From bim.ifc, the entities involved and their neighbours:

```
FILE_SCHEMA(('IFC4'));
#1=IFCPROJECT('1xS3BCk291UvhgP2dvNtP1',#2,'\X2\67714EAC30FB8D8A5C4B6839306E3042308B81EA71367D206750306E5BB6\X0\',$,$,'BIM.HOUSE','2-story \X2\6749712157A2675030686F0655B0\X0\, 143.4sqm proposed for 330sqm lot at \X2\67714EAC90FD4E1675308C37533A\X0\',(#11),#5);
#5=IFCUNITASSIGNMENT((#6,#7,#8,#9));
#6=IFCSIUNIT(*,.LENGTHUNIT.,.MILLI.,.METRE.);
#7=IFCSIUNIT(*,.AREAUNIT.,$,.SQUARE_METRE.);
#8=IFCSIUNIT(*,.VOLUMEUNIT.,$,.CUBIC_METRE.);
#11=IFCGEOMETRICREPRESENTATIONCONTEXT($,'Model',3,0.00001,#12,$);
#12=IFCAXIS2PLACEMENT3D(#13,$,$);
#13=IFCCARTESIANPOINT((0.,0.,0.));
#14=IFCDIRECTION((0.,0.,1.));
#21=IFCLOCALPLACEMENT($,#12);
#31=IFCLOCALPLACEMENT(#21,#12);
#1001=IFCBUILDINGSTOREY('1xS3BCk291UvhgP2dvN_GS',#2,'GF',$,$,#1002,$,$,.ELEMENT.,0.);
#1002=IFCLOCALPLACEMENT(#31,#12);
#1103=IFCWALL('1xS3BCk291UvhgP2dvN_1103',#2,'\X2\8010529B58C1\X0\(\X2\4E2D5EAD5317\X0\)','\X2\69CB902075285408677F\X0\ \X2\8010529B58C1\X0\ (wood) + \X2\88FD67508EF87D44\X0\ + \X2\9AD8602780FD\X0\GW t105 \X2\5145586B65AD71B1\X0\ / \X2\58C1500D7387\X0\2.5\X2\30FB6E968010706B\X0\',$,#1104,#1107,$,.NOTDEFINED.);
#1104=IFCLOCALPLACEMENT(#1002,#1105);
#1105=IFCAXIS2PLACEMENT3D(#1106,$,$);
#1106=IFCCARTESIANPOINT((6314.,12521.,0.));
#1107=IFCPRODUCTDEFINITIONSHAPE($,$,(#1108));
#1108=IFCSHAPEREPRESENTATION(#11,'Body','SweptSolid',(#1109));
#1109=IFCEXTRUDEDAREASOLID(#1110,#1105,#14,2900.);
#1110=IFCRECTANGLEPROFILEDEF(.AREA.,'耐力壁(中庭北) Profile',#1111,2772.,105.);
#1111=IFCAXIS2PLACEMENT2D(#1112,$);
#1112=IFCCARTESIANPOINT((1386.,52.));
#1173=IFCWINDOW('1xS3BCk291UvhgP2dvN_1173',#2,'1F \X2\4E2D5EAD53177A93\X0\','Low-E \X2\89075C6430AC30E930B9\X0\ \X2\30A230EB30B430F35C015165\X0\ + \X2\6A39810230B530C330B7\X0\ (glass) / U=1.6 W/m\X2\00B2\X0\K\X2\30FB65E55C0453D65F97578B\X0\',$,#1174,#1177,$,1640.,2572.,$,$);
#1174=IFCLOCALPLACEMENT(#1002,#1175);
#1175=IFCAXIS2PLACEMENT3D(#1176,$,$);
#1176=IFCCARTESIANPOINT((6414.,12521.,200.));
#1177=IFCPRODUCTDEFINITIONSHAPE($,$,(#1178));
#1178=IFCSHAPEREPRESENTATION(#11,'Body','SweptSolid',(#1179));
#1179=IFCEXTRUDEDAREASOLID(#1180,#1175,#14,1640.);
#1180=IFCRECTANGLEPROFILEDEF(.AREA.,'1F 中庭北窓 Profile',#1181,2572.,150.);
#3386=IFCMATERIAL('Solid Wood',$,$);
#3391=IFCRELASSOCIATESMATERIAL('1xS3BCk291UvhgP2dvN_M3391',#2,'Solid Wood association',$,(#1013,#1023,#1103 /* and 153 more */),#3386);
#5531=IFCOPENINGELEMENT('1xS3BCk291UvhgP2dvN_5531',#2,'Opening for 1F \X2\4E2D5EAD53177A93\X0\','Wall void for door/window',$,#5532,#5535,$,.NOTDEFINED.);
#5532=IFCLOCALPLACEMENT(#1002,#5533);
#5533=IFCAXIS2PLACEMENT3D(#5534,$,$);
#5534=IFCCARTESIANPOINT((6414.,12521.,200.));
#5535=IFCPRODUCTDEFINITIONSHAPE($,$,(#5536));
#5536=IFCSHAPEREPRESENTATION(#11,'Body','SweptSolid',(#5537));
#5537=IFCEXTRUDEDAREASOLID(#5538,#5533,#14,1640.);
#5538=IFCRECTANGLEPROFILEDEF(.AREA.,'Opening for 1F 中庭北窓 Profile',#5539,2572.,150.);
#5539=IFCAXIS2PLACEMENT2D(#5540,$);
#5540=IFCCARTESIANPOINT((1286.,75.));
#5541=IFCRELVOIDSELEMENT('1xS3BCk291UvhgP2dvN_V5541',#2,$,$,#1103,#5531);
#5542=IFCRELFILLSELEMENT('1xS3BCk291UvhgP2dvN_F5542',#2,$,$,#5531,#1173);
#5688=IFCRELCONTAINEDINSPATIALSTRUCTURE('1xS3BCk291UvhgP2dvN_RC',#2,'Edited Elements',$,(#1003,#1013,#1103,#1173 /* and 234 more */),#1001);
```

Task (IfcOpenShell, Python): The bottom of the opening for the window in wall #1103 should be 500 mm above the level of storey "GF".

```python
import numpy as np
import ifcopenshell
import ifcopenshell.api.geometry
import ifcopenshell.geom
import ifcopenshell.util.element
import ifcopenshell.util.placement
import ifcopenshell.util.shape
import ifcopenshell.util.unit

model = ifcopenshell.open("bim.ifc")
unit_scale = ifcopenshell.util.unit.calculate_unit_scale(model)

window = model.by_guid("1xS3BCk291UvhgP2dvN_1173")
opening = window.FillsVoids[0].RelatingOpeningElement
storey = ifcopenshell.util.element.get_container(window, ifc_class="IfcBuildingStorey")
level = ifcopenshell.util.placement.get_local_placement(storey.ObjectPlacement)[2, 3]

# The opening's origin need not be at the sill, so measure its lowest point.
shape = ifcopenshell.geom.create_shape(ifcopenshell.geom.settings(), opening)
bottom = ifcopenshell.util.shape.get_shape_bottom_elevation(shape, shape.geometry) / unit_scale
dz = level + 0.5 / unit_scale - bottom

shift = np.array([0.0, 0.0, dz])
# The window is not placed relative to its opening, so move both.
for product in (opening, window):
    matrix = ifcopenshell.util.placement.get_local_placement(product.ObjectPlacement)
    matrix[:3, 3] += shift
    ifcopenshell.api.geometry.edit_object_placement(model, product=product, matrix=matrix, is_si=False)

print(f"moved by {dz * unit_scale:+.3f} m")

model.write("bim_v2.ifc")
```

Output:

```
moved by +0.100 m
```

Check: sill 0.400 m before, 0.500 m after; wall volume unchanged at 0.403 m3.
